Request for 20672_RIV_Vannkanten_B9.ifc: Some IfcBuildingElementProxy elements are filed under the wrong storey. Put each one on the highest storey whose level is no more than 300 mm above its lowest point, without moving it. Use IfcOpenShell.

First a look at what the model holds.

```python
import ifcopenshell
import ifcopenshell.util.element
import ifcopenshell.util.placement

model = ifcopenshell.open("20672_RIV_Vannkanten_B9.ifc")
print(model.schema)
for storey in model.by_type("IfcBuildingStorey"):
    level = ifcopenshell.util.placement.get_storey_elevation(storey)
    count = sum(e.is_a("IfcBuildingElementProxy") for e in ifcopenshell.util.element.get_contained(storey))
    print(storey.id(), storey.Name, round(level, 3), count, sep=" | ")
```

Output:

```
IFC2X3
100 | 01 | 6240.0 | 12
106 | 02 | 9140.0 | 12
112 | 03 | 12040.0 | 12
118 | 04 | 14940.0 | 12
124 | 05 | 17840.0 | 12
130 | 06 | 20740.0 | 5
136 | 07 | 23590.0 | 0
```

```python
import ifcopenshell
import ifcopenshell.api.spatial
import ifcopenshell.geom
import ifcopenshell.util.element
import ifcopenshell.util.placement
import ifcopenshell.util.shape
import ifcopenshell.util.unit

model = ifcopenshell.open("20672_RIV_Vannkanten_B9.ifc")
unit_scale = ifcopenshell.util.unit.calculate_unit_scale(model)
settings = ifcopenshell.geom.settings()

levels = sorted(
    ((ifcopenshell.util.placement.get_storey_elevation(s) * unit_scale, s) for s in model.by_type("IfcBuildingStorey")),
    key=lambda pair: pair[0],
)

for e in model.by_type("IfcBuildingElementProxy"):
    current = e.ContainedInStructure[0].RelatingStructure if e.ContainedInStructure else None
    if current is None or not current.is_a("IfcBuildingStorey"):
        continue
    shape = ifcopenshell.geom.create_shape(settings, e)
    bottom = ifcopenshell.util.shape.get_shape_bottom_elevation(shape, shape.geometry)
    below = [s for level, s in levels if level <= bottom + 0.3]
    storey = below[-1] if below else levels[0][1]
    if storey != current:
        # assign_container keeps the world position.
        ifcopenshell.api.spatial.assign_container(model, products=[e], relating_structure=storey)
        print(e.id(), current.Name, "->", storey.Name)

model.write("20672_RIV_Vannkanten_B9_v2.ifc")
```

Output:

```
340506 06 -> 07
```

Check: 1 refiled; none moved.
